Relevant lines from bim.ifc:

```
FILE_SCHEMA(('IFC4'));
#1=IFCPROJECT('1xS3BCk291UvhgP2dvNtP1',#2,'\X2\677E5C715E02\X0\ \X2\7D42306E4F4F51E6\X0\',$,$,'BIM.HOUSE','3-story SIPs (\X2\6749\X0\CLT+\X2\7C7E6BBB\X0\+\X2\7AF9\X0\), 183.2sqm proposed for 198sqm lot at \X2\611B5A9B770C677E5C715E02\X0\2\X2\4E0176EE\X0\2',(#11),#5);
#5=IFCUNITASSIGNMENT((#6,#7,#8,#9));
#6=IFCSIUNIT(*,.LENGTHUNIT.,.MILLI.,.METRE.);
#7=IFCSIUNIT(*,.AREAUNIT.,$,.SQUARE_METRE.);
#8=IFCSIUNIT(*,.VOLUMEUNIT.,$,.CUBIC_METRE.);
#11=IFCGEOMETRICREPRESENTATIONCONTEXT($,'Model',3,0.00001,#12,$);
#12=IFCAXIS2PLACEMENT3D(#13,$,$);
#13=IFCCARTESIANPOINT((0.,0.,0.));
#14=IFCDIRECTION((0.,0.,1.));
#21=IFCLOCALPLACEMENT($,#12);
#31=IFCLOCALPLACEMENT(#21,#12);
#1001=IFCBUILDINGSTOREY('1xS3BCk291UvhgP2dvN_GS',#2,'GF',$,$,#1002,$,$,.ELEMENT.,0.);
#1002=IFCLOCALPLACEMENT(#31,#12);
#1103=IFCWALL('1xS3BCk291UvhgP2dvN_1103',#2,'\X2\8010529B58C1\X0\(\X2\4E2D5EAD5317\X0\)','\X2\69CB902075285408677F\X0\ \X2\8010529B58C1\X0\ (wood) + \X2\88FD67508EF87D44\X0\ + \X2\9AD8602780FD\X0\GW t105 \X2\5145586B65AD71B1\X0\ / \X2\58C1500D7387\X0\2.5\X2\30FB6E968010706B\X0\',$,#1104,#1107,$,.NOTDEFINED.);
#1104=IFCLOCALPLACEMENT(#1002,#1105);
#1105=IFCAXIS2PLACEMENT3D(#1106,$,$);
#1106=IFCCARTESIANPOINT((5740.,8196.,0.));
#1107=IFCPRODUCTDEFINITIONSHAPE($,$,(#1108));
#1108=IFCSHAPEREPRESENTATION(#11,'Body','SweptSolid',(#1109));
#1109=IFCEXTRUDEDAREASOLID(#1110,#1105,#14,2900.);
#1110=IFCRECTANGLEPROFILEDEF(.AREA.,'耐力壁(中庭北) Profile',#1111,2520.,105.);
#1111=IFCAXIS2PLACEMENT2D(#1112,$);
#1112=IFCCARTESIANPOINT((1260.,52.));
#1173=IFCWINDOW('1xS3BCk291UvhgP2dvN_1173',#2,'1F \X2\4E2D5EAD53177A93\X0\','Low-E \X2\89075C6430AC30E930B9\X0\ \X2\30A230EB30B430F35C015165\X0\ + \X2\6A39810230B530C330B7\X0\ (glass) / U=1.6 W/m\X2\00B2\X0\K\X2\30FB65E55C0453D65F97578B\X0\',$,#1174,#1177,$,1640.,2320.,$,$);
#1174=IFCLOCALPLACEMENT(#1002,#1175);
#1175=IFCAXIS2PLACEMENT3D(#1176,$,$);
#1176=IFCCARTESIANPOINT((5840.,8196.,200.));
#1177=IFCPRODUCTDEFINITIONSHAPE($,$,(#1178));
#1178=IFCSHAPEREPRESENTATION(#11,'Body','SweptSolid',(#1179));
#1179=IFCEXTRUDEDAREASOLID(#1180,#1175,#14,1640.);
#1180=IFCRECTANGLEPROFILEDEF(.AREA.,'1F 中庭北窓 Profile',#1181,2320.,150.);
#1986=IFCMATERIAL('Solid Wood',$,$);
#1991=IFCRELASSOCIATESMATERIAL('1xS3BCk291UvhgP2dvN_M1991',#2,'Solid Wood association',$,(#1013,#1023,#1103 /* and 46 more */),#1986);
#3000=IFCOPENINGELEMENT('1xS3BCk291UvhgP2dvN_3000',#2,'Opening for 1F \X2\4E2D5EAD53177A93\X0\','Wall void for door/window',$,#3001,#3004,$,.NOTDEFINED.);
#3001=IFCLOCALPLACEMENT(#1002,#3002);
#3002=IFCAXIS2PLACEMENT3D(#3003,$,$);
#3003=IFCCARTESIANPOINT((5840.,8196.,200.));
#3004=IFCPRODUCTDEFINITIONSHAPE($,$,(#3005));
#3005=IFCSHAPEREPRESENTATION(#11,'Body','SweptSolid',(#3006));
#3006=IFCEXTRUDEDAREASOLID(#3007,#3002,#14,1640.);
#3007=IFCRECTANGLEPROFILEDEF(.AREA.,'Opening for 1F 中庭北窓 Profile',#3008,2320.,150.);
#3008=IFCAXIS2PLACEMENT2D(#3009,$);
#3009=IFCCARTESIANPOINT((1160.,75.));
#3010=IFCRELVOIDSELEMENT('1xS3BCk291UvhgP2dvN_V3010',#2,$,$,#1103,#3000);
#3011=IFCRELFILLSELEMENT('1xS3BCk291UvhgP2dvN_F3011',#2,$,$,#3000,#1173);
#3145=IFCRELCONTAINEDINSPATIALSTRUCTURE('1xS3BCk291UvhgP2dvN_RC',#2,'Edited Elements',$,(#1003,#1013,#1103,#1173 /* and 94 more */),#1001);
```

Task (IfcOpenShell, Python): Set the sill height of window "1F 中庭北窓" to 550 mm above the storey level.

```python
import numpy as np
import ifcopenshell
import ifcopenshell.api.geometry
import ifcopenshell.geom
import ifcopenshell.util.element
import ifcopenshell.util.placement
import ifcopenshell.util.shape
import ifcopenshell.util.unit

model = ifcopenshell.open("bim.ifc")
unit_scale = ifcopenshell.util.unit.calculate_unit_scale(model)

window = model.by_id(1173)
opening = window.FillsVoids[0].RelatingOpeningElement
storey = ifcopenshell.util.element.get_container(window, ifc_class="IfcBuildingStorey")
level = ifcopenshell.util.placement.get_local_placement(storey.ObjectPlacement)[2, 3]

# The opening's origin need not be at the sill, so measure its lowest point.
shape = ifcopenshell.geom.create_shape(ifcopenshell.geom.settings(), opening)
bottom = ifcopenshell.util.shape.get_shape_bottom_elevation(shape, shape.geometry) / unit_scale
dz = level + 0.55 / unit_scale - bottom

shift = np.array([0.0, 0.0, dz])
# The window is not placed relative to its opening, so move both.
for product in (opening, window):
    matrix = ifcopenshell.util.placement.get_local_placement(product.ObjectPlacement)
    matrix[:3, 3] += shift
    ifcopenshell.api.geometry.edit_object_placement(model, product=product, matrix=matrix, is_si=False)

print(f"moved by {dz * unit_scale:+.3f} m")

model.write("bim-out.ifc")
```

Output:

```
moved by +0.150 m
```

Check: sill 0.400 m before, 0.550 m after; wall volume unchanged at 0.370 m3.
